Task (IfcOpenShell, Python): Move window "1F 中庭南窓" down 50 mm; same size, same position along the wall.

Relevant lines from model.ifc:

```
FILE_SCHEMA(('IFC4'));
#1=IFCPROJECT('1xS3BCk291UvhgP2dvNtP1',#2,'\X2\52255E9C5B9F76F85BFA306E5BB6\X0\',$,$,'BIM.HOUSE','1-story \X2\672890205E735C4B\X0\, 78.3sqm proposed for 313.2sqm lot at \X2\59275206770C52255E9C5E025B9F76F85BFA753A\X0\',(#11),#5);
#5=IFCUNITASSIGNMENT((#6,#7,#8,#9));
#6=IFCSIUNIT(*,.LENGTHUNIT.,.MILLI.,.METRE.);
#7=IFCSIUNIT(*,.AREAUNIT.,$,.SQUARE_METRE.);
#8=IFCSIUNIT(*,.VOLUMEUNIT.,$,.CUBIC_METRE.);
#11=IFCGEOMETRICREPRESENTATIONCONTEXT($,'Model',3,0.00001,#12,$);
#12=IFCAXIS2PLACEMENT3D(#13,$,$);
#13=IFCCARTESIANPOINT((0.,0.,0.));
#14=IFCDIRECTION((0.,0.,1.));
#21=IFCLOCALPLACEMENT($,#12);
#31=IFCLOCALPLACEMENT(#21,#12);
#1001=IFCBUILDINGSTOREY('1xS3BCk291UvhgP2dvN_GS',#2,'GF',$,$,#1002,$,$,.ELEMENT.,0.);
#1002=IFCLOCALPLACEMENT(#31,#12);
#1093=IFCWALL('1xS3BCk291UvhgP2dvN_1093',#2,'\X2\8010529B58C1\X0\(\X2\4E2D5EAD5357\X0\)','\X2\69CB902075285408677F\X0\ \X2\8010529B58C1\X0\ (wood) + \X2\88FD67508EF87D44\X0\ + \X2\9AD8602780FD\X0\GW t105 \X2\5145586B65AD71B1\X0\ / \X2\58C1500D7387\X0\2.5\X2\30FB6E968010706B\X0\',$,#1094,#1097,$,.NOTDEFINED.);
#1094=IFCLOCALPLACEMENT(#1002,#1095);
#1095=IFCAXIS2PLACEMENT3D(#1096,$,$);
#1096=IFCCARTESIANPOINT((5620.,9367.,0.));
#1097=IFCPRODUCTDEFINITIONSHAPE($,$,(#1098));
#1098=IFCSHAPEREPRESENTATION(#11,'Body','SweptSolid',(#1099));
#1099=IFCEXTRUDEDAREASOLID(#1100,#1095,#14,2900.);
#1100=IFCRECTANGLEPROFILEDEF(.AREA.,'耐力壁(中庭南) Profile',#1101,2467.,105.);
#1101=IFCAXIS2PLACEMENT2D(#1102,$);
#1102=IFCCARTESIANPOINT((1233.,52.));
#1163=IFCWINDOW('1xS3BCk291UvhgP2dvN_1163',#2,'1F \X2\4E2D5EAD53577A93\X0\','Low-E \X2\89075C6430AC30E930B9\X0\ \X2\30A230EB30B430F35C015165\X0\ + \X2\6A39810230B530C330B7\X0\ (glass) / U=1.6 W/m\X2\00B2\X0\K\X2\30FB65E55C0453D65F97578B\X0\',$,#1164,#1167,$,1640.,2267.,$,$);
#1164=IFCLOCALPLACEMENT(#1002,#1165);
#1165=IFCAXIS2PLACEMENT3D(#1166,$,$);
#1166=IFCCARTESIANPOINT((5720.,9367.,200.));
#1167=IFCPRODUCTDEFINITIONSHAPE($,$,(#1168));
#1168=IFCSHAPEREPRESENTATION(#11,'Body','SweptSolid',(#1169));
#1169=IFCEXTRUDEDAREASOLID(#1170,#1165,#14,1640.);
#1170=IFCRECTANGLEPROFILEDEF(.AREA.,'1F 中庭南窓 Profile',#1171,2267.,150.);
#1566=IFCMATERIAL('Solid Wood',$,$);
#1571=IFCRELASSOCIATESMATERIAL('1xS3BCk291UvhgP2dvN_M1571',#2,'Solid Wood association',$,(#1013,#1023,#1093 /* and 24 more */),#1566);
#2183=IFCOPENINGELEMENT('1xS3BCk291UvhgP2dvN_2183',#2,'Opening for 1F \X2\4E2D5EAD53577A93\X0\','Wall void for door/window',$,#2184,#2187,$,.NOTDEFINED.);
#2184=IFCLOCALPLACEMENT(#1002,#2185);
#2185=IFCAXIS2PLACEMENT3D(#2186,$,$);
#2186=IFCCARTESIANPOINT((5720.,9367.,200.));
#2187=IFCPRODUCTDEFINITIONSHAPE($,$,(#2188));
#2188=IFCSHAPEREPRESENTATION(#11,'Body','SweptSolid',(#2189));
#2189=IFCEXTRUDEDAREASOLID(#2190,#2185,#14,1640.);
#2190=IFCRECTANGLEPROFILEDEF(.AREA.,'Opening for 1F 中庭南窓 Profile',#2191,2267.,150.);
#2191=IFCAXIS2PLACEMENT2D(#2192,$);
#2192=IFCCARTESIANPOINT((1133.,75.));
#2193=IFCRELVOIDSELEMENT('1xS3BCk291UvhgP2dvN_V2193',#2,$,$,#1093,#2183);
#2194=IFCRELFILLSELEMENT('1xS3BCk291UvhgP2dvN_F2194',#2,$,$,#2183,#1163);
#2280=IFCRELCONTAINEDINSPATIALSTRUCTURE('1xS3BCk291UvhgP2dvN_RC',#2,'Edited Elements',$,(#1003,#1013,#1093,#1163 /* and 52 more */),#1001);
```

```python
import numpy as np
import ifcopenshell
import ifcopenshell.api.geometry
import ifcopenshell.util.placement
import ifcopenshell.util.unit

model = ifcopenshell.open("model.ifc")
unit_scale = ifcopenshell.util.unit.calculate_unit_scale(model)

window = model.by_guid("1xS3BCk291UvhgP2dvN_1163")
opening = window.FillsVoids[0].RelatingOpeningElement
dz = -50.0

shift = np.array([0.0, 0.0, dz])
# The window is not placed relative to its opening, so move both.
for product in (opening, window):
    matrix = ifcopenshell.util.placement.get_local_placement(product.ObjectPlacement)
    matrix[:3, 3] += shift
    ifcopenshell.api.geometry.edit_object_placement(model, product=product, matrix=matrix, is_si=False)

print(f"moved by {dz * unit_scale:+.3f} m")

model.write("model_rev.ifc")
```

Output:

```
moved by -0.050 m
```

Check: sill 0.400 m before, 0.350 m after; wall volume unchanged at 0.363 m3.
